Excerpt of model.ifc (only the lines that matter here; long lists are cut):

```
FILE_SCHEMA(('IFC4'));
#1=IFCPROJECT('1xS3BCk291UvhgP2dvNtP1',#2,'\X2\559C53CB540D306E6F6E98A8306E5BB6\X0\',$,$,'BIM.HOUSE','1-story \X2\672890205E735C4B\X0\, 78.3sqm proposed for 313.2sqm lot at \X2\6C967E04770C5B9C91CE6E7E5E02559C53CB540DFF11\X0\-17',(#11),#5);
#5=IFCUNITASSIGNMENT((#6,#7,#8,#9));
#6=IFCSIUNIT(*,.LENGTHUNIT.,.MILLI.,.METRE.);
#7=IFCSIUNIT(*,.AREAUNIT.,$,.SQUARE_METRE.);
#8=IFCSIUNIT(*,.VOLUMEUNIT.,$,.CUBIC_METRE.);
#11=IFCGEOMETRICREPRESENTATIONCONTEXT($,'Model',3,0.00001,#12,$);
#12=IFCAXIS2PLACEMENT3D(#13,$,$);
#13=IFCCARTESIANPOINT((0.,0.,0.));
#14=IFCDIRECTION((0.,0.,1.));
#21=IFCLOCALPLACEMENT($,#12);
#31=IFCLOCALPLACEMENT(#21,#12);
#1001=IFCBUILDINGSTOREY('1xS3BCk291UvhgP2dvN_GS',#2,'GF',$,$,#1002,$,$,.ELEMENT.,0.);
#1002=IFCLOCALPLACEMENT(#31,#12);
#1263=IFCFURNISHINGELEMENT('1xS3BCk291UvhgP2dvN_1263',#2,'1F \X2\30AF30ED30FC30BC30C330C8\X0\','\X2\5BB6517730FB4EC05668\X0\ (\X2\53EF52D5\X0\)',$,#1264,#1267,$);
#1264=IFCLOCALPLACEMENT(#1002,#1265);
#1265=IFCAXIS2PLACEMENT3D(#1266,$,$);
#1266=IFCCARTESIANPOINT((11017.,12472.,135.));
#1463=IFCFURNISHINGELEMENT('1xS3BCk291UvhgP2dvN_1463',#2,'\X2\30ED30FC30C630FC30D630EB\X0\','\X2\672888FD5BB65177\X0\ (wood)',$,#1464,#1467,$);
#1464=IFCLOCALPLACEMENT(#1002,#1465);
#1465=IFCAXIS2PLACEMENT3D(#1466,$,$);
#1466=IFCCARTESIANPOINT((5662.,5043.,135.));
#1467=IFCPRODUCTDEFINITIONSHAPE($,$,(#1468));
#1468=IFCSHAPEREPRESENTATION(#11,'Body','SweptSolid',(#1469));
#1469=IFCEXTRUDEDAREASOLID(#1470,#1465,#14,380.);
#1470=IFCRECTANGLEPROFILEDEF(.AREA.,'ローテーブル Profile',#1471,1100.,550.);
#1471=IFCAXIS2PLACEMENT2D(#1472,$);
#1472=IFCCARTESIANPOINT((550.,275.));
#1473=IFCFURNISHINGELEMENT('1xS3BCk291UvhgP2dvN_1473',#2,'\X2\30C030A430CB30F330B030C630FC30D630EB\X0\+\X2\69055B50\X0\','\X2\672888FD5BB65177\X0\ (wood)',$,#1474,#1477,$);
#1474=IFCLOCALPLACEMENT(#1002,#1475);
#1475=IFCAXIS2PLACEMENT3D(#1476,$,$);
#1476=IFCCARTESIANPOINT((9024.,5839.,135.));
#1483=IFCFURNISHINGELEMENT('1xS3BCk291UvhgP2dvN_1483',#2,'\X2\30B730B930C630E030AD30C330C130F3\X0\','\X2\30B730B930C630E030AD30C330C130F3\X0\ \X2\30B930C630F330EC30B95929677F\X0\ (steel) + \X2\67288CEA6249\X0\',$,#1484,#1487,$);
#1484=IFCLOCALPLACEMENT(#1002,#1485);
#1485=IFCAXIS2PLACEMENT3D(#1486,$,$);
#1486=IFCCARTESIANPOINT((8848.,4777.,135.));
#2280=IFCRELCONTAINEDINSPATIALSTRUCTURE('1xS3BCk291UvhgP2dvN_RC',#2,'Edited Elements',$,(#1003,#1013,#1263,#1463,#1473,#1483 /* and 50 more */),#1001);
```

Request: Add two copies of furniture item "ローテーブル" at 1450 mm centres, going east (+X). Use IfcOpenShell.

```python
import numpy as np
import ifcopenshell
import ifcopenshell.api.geometry
import ifcopenshell.api.root
import ifcopenshell.util.element
import ifcopenshell.util.placement
import ifcopenshell.util.unit

model = ifcopenshell.open("model.ifc")
unit_scale = ifcopenshell.util.unit.calculate_unit_scale(model)


def reuse_history(source, copy):
    """copy_class also copies each property set's owner history, people and application; keep the originals."""
    for rel in copy.IsDefinedBy:
        if rel.is_a("IfcRelDefinesByProperties") and (history := rel.RelatingPropertyDefinition.OwnerHistory):
            rel.RelatingPropertyDefinition.OwnerHistory = source.OwnerHistory
            ifcopenshell.util.element.remove_deep2(model, history)


source = model.by_guid("1xS3BCk291UvhgP2dvN_1463")
base = ifcopenshell.util.placement.get_local_placement(source.ObjectPlacement)
step = np.array([1.0, 0.0, 0.0]) * 1.45 / unit_scale

for i in range(1, 3):
    copy = ifcopenshell.api.root.copy_class(model, product=source)
    copy.Representation = ifcopenshell.util.element.copy_deep(
        model, source.Representation, exclude=["IfcGeometricRepresentationContext", "IfcRepresentationMap"]
    )
    reuse_history(source, copy)
    matrix = base.copy()
    matrix[:3, 3] += i * step
    print("added at", matrix[:3, 3].round(3) + 0.0)
    ifcopenshell.api.geometry.edit_object_placement(model, product=copy, matrix=matrix, is_si=False)

model.write("model_updated.ifc")
```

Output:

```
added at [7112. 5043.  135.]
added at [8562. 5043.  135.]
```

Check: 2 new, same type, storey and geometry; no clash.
